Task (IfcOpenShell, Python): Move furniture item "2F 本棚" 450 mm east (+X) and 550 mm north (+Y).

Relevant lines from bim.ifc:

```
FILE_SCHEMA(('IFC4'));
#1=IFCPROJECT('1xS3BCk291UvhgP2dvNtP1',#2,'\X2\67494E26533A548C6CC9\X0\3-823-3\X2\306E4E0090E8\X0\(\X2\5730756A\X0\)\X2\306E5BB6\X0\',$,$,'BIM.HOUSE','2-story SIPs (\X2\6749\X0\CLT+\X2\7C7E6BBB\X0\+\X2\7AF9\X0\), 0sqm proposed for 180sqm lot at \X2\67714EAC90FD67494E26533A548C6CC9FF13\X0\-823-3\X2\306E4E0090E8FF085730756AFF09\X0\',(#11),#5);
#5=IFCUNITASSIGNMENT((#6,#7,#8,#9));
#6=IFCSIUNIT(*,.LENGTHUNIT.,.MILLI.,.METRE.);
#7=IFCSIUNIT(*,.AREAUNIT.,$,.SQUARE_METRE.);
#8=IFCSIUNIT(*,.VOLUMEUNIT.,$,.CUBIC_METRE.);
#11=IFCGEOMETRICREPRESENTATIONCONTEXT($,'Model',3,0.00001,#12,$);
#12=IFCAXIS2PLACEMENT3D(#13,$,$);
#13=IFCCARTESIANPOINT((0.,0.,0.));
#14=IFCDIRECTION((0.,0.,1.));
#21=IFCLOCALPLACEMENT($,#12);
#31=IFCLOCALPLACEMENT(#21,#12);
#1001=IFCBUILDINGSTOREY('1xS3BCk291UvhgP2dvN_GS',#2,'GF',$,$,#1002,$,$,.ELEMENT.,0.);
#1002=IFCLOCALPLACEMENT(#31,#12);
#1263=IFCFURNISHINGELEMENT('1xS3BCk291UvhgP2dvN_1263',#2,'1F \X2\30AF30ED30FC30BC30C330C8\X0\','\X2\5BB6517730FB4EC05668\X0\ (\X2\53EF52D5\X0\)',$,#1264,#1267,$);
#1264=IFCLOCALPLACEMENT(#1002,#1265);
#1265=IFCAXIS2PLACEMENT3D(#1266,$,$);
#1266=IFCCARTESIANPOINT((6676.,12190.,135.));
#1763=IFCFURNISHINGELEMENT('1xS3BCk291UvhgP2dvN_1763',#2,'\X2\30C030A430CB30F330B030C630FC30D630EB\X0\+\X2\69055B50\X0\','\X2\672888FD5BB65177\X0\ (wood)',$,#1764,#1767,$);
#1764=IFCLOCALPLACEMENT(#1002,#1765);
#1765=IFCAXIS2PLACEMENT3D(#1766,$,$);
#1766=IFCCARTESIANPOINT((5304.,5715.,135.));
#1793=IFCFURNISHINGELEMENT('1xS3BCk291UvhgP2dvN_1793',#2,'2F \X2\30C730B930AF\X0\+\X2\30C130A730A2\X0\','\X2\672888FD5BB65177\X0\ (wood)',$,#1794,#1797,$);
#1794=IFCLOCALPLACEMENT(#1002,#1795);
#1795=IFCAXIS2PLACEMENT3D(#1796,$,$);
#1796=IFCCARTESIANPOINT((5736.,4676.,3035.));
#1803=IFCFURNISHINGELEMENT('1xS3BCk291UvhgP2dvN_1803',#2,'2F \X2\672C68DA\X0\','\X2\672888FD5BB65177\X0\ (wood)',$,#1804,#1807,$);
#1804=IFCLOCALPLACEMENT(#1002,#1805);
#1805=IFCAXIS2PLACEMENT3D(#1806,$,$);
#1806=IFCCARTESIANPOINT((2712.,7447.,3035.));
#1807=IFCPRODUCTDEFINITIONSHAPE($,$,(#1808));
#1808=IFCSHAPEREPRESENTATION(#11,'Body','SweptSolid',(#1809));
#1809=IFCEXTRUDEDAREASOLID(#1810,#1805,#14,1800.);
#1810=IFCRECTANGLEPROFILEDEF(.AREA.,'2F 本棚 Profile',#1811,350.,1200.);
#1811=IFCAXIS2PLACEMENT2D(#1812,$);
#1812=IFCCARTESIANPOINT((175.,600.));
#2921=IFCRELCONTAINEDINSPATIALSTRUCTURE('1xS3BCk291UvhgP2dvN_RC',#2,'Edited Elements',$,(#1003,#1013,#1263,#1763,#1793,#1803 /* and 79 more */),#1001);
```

```python
import ifcopenshell
import ifcopenshell.api.geometry
import ifcopenshell.util.placement
import ifcopenshell.util.unit

model = ifcopenshell.open("bim.ifc")
unit_scale = ifcopenshell.util.unit.calculate_unit_scale(model)

item = model.by_guid("1xS3BCk291UvhgP2dvN_1803")
matrix = ifcopenshell.util.placement.get_local_placement(item.ObjectPlacement)
matrix[0, 3] += 0.45 / unit_scale
matrix[1, 3] += 0.55 / unit_scale
ifcopenshell.api.geometry.edit_object_placement(model, product=item, matrix=matrix, is_si=False)

print(ifcopenshell.util.placement.get_local_placement(item.ObjectPlacement).round(3) + 0.0)

model.write("bim_rev.ifc")
```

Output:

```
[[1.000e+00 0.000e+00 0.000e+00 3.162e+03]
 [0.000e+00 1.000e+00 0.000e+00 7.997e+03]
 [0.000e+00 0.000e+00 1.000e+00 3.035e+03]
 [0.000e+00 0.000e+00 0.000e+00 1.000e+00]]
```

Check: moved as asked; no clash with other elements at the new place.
